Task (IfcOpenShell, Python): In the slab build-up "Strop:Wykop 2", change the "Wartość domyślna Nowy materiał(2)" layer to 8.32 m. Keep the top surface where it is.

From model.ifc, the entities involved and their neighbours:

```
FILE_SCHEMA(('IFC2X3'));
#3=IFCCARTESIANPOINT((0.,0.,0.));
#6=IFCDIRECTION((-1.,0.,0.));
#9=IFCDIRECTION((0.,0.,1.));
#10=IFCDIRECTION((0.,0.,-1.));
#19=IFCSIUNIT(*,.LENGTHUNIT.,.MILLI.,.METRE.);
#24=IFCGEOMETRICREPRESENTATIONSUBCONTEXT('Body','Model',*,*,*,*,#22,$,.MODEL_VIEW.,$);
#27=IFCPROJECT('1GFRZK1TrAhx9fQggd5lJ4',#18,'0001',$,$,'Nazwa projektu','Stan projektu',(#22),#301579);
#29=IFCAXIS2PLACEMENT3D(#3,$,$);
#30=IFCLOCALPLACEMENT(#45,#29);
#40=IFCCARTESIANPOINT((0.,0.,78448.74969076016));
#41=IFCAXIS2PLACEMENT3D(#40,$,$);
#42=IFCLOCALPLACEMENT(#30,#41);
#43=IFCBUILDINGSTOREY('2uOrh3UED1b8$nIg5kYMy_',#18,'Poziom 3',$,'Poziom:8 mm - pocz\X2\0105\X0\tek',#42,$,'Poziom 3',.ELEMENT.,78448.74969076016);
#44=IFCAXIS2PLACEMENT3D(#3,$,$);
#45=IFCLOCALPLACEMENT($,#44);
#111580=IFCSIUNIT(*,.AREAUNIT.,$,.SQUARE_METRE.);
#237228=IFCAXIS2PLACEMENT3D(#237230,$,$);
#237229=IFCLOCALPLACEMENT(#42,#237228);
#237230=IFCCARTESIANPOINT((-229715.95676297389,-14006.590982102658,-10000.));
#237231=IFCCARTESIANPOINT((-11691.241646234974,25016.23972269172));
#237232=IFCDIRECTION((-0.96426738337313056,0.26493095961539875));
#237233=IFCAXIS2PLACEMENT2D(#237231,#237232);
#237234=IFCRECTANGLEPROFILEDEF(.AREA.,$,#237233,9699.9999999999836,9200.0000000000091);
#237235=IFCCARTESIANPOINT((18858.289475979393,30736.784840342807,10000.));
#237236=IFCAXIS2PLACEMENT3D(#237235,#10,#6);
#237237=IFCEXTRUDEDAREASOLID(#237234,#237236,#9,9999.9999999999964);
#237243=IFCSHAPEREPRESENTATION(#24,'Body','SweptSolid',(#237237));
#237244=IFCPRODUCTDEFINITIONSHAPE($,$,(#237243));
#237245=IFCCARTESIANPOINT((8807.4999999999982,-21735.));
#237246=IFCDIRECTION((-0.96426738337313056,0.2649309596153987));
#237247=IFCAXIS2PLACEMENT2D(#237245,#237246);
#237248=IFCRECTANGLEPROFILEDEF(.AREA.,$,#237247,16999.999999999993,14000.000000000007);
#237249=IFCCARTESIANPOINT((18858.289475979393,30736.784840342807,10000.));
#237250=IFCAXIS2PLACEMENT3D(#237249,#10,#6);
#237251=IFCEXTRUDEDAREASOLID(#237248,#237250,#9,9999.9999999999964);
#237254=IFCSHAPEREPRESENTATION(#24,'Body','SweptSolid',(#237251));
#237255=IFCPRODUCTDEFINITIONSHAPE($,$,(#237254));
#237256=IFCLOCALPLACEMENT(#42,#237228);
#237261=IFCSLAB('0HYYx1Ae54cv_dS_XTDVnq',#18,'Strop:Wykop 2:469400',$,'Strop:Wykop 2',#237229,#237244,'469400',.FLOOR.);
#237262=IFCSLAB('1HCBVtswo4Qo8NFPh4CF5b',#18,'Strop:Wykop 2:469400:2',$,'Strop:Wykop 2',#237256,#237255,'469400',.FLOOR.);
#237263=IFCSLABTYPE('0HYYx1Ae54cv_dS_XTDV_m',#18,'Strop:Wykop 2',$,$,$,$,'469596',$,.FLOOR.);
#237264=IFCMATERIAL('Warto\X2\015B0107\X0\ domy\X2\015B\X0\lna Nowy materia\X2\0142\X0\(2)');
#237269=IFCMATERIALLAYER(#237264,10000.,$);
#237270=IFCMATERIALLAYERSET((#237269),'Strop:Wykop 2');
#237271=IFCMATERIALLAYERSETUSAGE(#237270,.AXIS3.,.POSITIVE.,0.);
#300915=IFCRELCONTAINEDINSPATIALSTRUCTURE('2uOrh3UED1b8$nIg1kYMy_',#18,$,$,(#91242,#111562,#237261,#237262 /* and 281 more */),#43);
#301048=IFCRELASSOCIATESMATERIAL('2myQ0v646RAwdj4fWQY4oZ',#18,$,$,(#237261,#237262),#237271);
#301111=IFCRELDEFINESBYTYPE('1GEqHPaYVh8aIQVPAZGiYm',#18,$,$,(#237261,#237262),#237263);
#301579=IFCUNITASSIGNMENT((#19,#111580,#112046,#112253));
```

```python
import ifcopenshell
import ifcopenshell.util.element
import ifcopenshell.util.representation

model = ifcopenshell.open("model.ifc")

layer_set = model.by_id(237270)
layer = next(l for l in layer_set.MaterialLayers if l.Material and l.Material.Name == "Wartość domyślna Nowy materiał(2)")
change = 8320.0 - layer.LayerThickness
layer.LayerThickness += change

# The layer set is shared, so every slab that uses it gets the new thickness.
slabs = [e for e in ifcopenshell.util.element.get_elements_by_material(model, layer_set) if e.is_a("IfcSlab")]
for slab in sorted(slabs, key=lambda e: e.id()):
    body = ifcopenshell.util.representation.get_representation(slab, "Model", "Body")
    solid = body.Items[0]
    old_depth = solid.Depth
    solid.Depth += change
    print(slab.id(), f"{old_depth:g} -> {solid.Depth:g}")

# The layers are counted up from the underside, which has moved.
for usage in {ifcopenshell.util.element.get_material(slab) for slab in slabs}:
    usage.OffsetFromReferenceLine -= change

model.write("model_v2.ifc")
```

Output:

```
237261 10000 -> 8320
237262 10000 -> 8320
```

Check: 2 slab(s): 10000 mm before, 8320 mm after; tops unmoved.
